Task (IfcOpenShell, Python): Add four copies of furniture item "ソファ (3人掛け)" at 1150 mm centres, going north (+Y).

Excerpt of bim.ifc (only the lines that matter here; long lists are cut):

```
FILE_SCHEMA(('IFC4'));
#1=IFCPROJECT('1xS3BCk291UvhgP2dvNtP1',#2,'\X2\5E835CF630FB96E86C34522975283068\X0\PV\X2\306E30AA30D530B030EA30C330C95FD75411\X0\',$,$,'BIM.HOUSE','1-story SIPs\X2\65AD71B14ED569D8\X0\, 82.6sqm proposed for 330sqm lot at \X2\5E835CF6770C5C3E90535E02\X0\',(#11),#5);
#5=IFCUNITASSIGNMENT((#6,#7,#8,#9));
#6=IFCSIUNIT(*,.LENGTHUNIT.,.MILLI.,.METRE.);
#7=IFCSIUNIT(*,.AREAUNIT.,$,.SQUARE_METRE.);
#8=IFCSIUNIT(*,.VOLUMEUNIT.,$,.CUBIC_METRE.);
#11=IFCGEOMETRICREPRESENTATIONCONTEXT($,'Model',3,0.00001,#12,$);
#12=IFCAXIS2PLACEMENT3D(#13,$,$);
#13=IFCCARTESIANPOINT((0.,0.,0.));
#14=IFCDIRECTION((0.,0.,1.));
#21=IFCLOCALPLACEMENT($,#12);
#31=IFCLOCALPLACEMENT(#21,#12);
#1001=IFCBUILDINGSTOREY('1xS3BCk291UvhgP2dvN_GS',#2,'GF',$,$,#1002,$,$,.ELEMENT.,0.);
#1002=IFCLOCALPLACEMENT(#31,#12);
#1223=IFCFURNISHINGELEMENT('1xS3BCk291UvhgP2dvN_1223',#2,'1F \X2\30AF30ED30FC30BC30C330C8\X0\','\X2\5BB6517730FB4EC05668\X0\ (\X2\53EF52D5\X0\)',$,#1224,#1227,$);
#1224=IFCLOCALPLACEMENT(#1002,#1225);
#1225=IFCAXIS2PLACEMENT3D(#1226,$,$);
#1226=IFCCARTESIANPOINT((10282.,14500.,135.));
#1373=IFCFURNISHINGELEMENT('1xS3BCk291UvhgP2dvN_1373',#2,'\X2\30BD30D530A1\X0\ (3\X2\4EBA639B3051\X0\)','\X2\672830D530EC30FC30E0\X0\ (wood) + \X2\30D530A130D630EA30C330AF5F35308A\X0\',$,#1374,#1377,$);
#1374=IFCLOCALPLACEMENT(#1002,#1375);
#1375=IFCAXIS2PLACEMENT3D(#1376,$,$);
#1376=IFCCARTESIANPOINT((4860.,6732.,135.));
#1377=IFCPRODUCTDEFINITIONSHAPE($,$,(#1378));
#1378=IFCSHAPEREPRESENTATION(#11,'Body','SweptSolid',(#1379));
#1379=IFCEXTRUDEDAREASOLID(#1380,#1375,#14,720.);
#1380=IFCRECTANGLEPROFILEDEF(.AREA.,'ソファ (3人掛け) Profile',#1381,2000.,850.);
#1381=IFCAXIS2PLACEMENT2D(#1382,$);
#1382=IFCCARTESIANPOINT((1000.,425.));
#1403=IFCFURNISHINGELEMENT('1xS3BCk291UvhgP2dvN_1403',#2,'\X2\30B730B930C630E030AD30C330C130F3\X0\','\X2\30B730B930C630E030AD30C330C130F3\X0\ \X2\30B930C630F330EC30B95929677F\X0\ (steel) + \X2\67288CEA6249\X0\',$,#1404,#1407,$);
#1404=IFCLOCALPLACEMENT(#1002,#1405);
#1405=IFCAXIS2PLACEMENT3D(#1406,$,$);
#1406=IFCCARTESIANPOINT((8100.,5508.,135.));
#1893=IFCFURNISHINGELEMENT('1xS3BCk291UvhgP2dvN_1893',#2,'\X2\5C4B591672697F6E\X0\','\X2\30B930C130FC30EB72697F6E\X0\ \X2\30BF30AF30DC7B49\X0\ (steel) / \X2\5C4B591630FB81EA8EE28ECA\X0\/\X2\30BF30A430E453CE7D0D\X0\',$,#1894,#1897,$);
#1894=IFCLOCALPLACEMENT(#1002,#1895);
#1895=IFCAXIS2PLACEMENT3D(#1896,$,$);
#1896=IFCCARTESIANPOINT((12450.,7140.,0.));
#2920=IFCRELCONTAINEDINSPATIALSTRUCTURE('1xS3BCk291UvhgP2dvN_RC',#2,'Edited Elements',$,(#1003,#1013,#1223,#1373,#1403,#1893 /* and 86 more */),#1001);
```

```python
import numpy as np
import ifcopenshell
import ifcopenshell.api.geometry
import ifcopenshell.api.root
import ifcopenshell.util.element
import ifcopenshell.util.placement

model = ifcopenshell.open("bim.ifc")


def reuse_history(source, copy):
    """copy_class also copies each property set's owner history, people and application; keep the originals."""
    for rel in copy.IsDefinedBy:
        if rel.is_a("IfcRelDefinesByProperties") and (history := rel.RelatingPropertyDefinition.OwnerHistory):
            rel.RelatingPropertyDefinition.OwnerHistory = source.OwnerHistory
            ifcopenshell.util.element.remove_deep2(model, history)


source = model.by_guid("1xS3BCk291UvhgP2dvN_1373")
base = ifcopenshell.util.placement.get_local_placement(source.ObjectPlacement)
step = np.array([0.0, 1.0, 0.0]) * 1150.0

for i in range(1, 5):
    copy = ifcopenshell.api.root.copy_class(model, product=source)
    copy.Representation = ifcopenshell.util.element.copy_deep(
        model, source.Representation, exclude=["IfcGeometricRepresentationContext", "IfcRepresentationMap"]
    )
    reuse_history(source, copy)
    matrix = base.copy()
    matrix[:3, 3] += i * step
    print("added at", matrix[:3, 3].round(3) + 0.0)
    ifcopenshell.api.geometry.edit_object_placement(model, product=copy, matrix=matrix, is_si=False)

model.write("bim_edited.ifc")
```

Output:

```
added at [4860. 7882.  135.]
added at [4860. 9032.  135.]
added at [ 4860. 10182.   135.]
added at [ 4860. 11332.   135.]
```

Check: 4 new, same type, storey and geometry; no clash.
